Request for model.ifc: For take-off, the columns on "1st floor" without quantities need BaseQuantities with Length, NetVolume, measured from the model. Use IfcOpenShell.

First a look at what the model holds.

```python
import ifcopenshell
import ifcopenshell.util.element
import ifcopenshell.util.unit

model = ifcopenshell.open("model.ifc")
print(model.schema)
for unit_type in ("LENGTHUNIT", "AREAUNIT", "VOLUMEUNIT"):
    print(unit_type, ifcopenshell.util.unit.calculate_unit_scale(model, unit_type))
storey = next(s for s in model.by_type("IfcBuildingStorey") if s.Name == "1st floor")
columns = [e for e in ifcopenshell.util.element.get_decomposition(storey) if e.is_a("IfcColumn")]
for e in sorted(columns, key=lambda e: e.id()):
    print(e.id(), e.is_a(), e.Name, list(ifcopenshell.util.element.get_psets(e, qtos_only=True)), sep=" | ")
```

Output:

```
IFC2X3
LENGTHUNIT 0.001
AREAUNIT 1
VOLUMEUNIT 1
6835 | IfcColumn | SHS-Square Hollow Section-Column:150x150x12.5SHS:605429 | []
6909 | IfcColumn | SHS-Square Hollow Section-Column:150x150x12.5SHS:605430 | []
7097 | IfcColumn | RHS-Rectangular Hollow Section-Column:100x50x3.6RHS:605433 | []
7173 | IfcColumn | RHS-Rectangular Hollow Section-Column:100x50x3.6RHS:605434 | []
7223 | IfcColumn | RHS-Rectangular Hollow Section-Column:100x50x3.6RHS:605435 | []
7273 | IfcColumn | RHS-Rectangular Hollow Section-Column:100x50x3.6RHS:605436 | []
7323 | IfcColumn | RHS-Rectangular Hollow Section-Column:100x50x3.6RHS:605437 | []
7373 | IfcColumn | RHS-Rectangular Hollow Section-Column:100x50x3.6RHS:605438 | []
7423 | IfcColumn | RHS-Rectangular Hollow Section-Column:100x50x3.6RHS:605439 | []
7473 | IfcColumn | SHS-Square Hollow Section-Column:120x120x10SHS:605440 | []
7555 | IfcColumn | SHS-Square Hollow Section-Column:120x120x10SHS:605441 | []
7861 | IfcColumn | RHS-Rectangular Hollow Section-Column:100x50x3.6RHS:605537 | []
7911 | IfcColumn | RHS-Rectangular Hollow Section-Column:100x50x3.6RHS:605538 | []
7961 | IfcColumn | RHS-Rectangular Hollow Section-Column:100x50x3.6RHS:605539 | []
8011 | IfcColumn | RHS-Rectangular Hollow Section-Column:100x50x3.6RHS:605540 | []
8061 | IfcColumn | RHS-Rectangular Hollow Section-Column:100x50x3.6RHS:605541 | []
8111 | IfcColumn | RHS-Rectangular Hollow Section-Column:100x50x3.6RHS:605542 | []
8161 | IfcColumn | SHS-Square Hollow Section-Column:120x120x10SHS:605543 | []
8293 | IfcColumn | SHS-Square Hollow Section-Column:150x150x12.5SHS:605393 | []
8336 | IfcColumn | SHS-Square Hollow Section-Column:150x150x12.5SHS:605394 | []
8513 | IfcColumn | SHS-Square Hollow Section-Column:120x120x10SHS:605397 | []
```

```python
import ifcopenshell
import ifcopenshell.api.pset
import ifcopenshell.geom
import ifcopenshell.util.element
import ifcopenshell.util.shape
import ifcopenshell.util.unit

model = ifcopenshell.open("model.ifc")
unit_scale = ifcopenshell.util.unit.calculate_unit_scale(model)
volume_scale = ifcopenshell.util.unit.calculate_unit_scale(model, "VOLUMEUNIT")
settings = ifcopenshell.geom.settings()

storey = next(s for s in model.by_type("IfcBuildingStorey") if s.Name == "1st floor")
columns = [e for e in ifcopenshell.util.element.get_decomposition(storey) if e.is_a("IfcColumn")]

for e in sorted(columns, key=lambda e: e.id()):
    if ifcopenshell.util.element.get_psets(e, qtos_only=True, should_inherit=False):
        continue
    # Geometry comes back in metres, in the element's own axes.
    shape = ifcopenshell.geom.create_shape(settings, e)
    values = {
        "Length": ifcopenshell.util.shape.get_z(shape.geometry) / unit_scale,
        "NetVolume": ifcopenshell.util.shape.get_volume(shape.geometry) / volume_scale,
    }
    qto = ifcopenshell.api.pset.add_qto(model, product=e, name="BaseQuantities")
    ifcopenshell.api.pset.edit_qto(model, qto=qto, properties=values)
    print(e.id(), {k: round(v, 3) for k, v in values.items()})

model.write("model_edited.ifc")
```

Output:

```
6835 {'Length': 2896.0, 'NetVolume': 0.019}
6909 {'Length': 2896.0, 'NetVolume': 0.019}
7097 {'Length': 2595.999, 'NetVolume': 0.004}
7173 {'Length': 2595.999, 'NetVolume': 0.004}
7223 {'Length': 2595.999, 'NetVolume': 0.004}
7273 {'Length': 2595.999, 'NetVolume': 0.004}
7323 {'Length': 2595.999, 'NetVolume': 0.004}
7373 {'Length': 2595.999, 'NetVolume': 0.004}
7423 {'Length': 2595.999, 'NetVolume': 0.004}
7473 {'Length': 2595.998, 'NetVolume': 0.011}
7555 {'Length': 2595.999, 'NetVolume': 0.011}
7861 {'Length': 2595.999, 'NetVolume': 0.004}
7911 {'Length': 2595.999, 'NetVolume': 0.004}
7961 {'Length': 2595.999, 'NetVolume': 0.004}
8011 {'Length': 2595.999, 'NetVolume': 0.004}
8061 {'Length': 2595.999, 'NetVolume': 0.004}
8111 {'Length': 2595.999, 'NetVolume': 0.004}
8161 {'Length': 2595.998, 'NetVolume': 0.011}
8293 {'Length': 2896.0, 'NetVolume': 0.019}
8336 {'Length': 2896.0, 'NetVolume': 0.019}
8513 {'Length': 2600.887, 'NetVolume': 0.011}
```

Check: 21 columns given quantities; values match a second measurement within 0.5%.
